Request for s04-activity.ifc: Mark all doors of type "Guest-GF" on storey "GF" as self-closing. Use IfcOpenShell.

First a look at what the model holds.

```python
import ifcopenshell
import ifcopenshell.util.element

model = ifcopenshell.open("s04-activity.ifc")
print(model.schema)
storey = next(s for s in model.by_type("IfcBuildingStorey") if s.Name == "GF")
doors = [e for e in ifcopenshell.util.element.get_decomposition(storey) if e.is_a("IfcDoor")]
seen = {}
for e in doors:
    element_type = ifcopenshell.util.element.get_type(e)
    key = (element_type.Name if element_type != e and element_type else None, ifcopenshell.util.element.get_pset(e, "Pset_DoorCommon", "SelfClosing"))
    seen[key] = seen.get(key, 0) + 1
for (name, value), count in sorted(seen.items(), key=str):
    print(count, "x", name, "|", value)
```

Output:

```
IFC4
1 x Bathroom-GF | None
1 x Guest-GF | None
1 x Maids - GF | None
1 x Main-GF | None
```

```python
import ifcopenshell
import ifcopenshell.api.pset
import ifcopenshell.util.element

model = ifcopenshell.open("s04-activity.ifc")

storey = next(s for s in model.by_type("IfcBuildingStorey") if s.Name == "GF")
doors = [e for e in ifcopenshell.util.element.get_decomposition(storey) if e.is_a("IfcDoor")]

count = 0
for e in doors:
    element_type = ifcopenshell.util.element.get_type(e)
    if element_type in (None, e) or element_type.Name != "Guest-GF":
        continue
    # add_pset returns the element's existing set when there is one.
    pset = ifcopenshell.api.pset.add_pset(model, product=e, name="Pset_DoorCommon")
    ifcopenshell.api.pset.edit_pset(model, pset=pset, properties={"SelfClosing": True})
    count += 1

print(count, "doors updated")

model.write("s04-activity-out.ifc")
```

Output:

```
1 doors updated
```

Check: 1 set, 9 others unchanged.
